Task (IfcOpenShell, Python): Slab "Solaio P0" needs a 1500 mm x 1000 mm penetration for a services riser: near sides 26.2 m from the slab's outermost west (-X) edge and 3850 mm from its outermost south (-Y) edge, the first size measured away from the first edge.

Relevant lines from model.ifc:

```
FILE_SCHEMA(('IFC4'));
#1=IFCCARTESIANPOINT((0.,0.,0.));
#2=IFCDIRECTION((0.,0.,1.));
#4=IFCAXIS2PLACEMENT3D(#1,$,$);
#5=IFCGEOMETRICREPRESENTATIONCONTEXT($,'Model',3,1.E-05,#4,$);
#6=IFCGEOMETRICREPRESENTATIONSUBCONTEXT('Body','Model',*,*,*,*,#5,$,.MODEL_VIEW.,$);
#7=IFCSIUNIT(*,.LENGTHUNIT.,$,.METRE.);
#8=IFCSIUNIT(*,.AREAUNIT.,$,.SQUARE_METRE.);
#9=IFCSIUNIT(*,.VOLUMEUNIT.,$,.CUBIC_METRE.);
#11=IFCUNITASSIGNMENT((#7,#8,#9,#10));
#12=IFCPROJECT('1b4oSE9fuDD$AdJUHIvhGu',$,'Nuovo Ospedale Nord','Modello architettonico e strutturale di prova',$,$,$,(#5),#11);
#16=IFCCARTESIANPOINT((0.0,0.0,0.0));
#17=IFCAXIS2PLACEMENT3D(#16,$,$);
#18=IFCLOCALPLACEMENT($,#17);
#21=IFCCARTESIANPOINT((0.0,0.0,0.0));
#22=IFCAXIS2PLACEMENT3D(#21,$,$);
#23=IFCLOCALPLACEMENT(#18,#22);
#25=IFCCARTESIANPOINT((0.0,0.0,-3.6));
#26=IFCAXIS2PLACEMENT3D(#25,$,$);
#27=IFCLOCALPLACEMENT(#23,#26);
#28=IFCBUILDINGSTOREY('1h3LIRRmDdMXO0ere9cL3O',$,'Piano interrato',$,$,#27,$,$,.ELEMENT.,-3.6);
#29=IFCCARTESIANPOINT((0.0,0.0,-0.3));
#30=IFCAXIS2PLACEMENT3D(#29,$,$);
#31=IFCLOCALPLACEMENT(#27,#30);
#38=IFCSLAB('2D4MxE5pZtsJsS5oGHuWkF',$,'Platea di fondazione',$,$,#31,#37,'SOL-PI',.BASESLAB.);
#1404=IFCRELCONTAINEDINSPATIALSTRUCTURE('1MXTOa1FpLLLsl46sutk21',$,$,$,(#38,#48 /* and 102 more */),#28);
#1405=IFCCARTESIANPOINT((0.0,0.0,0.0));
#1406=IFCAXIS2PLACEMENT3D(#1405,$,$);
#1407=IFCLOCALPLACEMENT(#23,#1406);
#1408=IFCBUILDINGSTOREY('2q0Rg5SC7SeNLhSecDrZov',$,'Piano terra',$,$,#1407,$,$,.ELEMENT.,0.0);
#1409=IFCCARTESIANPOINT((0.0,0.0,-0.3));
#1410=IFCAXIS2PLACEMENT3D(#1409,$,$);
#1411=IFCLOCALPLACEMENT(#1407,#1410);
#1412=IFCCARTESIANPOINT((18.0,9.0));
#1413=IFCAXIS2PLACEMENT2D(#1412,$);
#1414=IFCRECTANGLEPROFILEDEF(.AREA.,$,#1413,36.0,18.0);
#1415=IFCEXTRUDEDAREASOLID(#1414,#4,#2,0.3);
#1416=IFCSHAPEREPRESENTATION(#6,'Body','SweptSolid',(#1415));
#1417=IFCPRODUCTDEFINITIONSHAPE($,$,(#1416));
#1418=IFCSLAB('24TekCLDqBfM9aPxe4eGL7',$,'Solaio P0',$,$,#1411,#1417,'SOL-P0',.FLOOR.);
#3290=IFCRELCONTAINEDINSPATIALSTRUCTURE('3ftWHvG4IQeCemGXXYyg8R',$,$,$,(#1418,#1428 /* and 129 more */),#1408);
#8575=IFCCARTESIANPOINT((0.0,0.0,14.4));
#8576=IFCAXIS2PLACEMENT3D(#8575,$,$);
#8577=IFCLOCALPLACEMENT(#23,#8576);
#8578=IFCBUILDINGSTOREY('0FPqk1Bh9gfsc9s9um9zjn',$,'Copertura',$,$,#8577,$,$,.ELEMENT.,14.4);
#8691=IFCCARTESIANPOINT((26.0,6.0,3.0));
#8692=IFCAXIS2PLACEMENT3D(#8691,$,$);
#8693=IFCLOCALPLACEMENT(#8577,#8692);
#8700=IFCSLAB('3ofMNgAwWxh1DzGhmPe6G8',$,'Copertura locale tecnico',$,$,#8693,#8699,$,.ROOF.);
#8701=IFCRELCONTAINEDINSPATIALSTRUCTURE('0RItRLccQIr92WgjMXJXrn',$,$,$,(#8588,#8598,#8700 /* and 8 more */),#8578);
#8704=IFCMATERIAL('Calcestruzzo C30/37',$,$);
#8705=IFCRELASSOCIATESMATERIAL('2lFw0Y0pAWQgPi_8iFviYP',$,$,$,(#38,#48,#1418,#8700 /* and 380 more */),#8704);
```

```python
import numpy as np
import ifcopenshell
import ifcopenshell.api.feature
import ifcopenshell.api.geometry
import ifcopenshell.api.root
import ifcopenshell.geom
import ifcopenshell.util.placement
import ifcopenshell.util.representation
import ifcopenshell.util.shape
import ifcopenshell.util.unit

model = ifcopenshell.open("model.ifc")
unit_scale = ifcopenshell.util.unit.calculate_unit_scale(model)
settings = ifcopenshell.geom.settings()


def volume(element):
    """Net volume in cubic metres, openings subtracted."""
    shape = ifcopenshell.geom.create_shape(settings, element)
    return ifcopenshell.util.shape.get_volume(shape.geometry)


slab = model.by_guid("24TekCLDqBfM9aPxe4eGL7")
before = volume(slab)

# Extent in the slab's own axes, in metres. The edges named are its -X and -Y sides.
slab_shape = ifcopenshell.geom.create_shape(settings, slab)
vertices = ifcopenshell.util.shape.get_vertices(slab_shape.geometry)
x_min, y_min, bottom = vertices.min(axis=0)
top = vertices[:, 2].max()

opening = ifcopenshell.api.root.create_entity(model, ifc_class="IfcOpeningElement", name="Services riser opening", predefined_type="OPENING")
context = ifcopenshell.util.representation.get_context(model, "Model", "Body", "MODEL_VIEW")
width, depth = 1.5, 1
outline = [(0.0, 0.0), (width, 0.0), (width, depth), (0.0, depth), (0.0, 0.0)]
# Overshoot both faces by 50 mm so the cut is clean.
shape = ifcopenshell.api.geometry.add_slab_representation(
    model, context=context, depth=top - bottom + 0.1, polyline=outline
)
ifcopenshell.api.geometry.assign_representation(model, product=opening, representation=shape)

matrix = ifcopenshell.util.placement.get_local_placement(slab.ObjectPlacement)
matrix[:, 3] = matrix @ np.append(np.array([x_min + 26.2, y_min + 3.85, bottom - 0.05]) / unit_scale, 1.0)
ifcopenshell.api.geometry.edit_object_placement(model, product=opening, matrix=matrix, is_si=False)
ifcopenshell.api.feature.add_feature(model, feature=opening, element=slab)

after = volume(slab)

print(f"slab volume {before:.3f} -> {after:.3f} m3")

model.write("model-out.ifc")
```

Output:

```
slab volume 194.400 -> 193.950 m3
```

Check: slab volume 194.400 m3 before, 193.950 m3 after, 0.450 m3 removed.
